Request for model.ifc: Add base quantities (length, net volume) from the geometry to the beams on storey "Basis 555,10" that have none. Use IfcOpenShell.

First a look at what the model holds.

```python
import ifcopenshell
import ifcopenshell.util.element
import ifcopenshell.util.unit

model = ifcopenshell.open("model.ifc")
print(model.schema)
for unit_type in ("LENGTHUNIT", "AREAUNIT", "VOLUMEUNIT"):
    print(unit_type, ifcopenshell.util.unit.calculate_unit_scale(model, unit_type))
storey = next(s for s in model.by_type("IfcBuildingStorey") if s.Name == "Basis 555,10")
beams = [e for e in ifcopenshell.util.element.get_decomposition(storey) if e.is_a("IfcBeam")]
for e in sorted(beams, key=lambda e: e.id()):
    print(e.id(), e.is_a(), e.Name, list(ifcopenshell.util.element.get_psets(e, qtos_only=True)), sep=" | ")
```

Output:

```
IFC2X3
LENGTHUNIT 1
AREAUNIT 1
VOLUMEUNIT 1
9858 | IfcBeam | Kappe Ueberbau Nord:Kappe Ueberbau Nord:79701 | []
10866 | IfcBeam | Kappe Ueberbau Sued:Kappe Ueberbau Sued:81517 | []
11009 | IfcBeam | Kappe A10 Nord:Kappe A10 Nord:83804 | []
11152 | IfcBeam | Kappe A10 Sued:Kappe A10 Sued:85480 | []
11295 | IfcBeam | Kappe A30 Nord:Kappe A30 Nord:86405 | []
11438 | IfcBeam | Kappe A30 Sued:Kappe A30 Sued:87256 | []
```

```python
import ifcopenshell
import ifcopenshell.api.pset
import ifcopenshell.geom
import ifcopenshell.util.element
import ifcopenshell.util.shape
import ifcopenshell.util.unit

model = ifcopenshell.open("model.ifc")
unit_scale = ifcopenshell.util.unit.calculate_unit_scale(model)
volume_scale = ifcopenshell.util.unit.calculate_unit_scale(model, "VOLUMEUNIT")
settings = ifcopenshell.geom.settings()

storey = next(s for s in model.by_type("IfcBuildingStorey") if s.Name == "Basis 555,10")
beams = [e for e in ifcopenshell.util.element.get_decomposition(storey) if e.is_a("IfcBeam")]

for e in sorted(beams, key=lambda e: e.id()):
    if ifcopenshell.util.element.get_psets(e, qtos_only=True, should_inherit=False):
        continue
    # Geometry comes back in metres, in the element's own axes.
    shape = ifcopenshell.geom.create_shape(settings, e)
    values = {
        "Length": ifcopenshell.util.shape.get_max_xyz(shape.geometry) / unit_scale,
        "NetVolume": ifcopenshell.util.shape.get_volume(shape.geometry) / volume_scale,
    }
    qto = ifcopenshell.api.pset.add_qto(model, product=e, name="BaseQuantities")
    ifcopenshell.api.pset.edit_qto(model, qto=qto, properties=values)
    print(e.id(), {k: round(v, 3) for k, v in values.items()})

model.write("model_v2.ifc")
```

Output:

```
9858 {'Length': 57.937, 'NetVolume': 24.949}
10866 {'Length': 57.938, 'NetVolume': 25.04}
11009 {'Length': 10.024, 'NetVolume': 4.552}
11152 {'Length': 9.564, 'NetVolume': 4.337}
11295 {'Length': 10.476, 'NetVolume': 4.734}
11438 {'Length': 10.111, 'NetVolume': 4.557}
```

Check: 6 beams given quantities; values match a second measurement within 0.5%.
